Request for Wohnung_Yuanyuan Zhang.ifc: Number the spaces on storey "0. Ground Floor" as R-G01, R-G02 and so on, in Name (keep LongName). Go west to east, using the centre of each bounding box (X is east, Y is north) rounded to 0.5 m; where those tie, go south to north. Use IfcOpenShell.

First a look at what the model holds.

```python
import ifcopenshell
import ifcopenshell.util.element
import ifcopenshell.util.placement

model = ifcopenshell.open("Wohnung_Yuanyuan Zhang.ifc")
print(model.schema)
storey = next(s for s in model.by_type("IfcBuildingStorey") if s.Name == "0. Ground Floor")
spaces = [e for e in ifcopenshell.util.element.get_decomposition(storey) if e.is_a("IfcSpace")]
for e in sorted(spaces, key=lambda e: e.id()):
    origin = ifcopenshell.util.placement.get_local_placement(e.ObjectPlacement)[:3, 3]
    print(e.id(), e.Name, e.LongName, origin.round(2) + 0.0, sep=" | ")
```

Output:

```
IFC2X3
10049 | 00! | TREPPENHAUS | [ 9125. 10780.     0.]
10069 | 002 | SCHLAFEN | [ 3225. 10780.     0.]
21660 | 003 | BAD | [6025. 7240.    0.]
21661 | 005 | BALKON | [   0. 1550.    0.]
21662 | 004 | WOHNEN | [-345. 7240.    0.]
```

```python
import ifcopenshell
import ifcopenshell.geom
import ifcopenshell.util.element
import ifcopenshell.util.shape

model = ifcopenshell.open("Wohnung_Yuanyuan Zhang.ifc")
settings = ifcopenshell.geom.settings()
settings.set("use-world-coords", True)


def centre(element):
    shape = ifcopenshell.geom.create_shape(settings, element)
    return ifcopenshell.util.shape.get_bbox_centroid(shape.geometry)


storey = next(s for s in model.by_type("IfcBuildingStorey") if s.Name == "0. Ground Floor")
spaces = [e for e in ifcopenshell.util.element.get_decomposition(storey) if e.is_a("IfcSpace")]

# Insertion points can sit at a corner or the storey origin, so sort by the geometry (in metres).
centres = {e: centre(e) for e in spaces}
spaces.sort(key=lambda e: (round(centres[e][0] / 0.5), centres[e][1]))

for i, e in enumerate(spaces, start=1):
    number = f"R-G{i:02d}"
    e.Name = number
    print(e.id(), number)

model.write("Wohnung_Yuanyuan Zhang_updated.ifc")
```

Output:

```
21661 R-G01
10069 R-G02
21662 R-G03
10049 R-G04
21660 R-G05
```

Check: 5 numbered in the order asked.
